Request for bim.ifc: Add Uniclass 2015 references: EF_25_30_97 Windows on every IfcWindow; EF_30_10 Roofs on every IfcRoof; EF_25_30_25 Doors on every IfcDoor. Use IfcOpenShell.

First a look at what the model holds.

```python
import ifcopenshell

model = ifcopenshell.open("bim.ifc")
print(model.schema)
print("classifications:", [c.Name for c in model.by_type("IfcClassification")])
for ifc_class in ("IfcDoor", "IfcRoof", "IfcStair", "IfcWall", "IfcWindow"):
    print(ifc_class, len(model.by_type(ifc_class)))
```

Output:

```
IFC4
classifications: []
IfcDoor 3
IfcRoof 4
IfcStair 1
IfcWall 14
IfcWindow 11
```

```python
import ifcopenshell
import ifcopenshell.api.classification

model = ifcopenshell.open("bim.ifc")

system = ifcopenshell.api.classification.add_classification(model, classification="Uniclass 2015")

codes = {
    "IfcWindow": ("EF_25_30_97", "Windows"),
    "IfcRoof": ("EF_30_10", "Roofs"),
    "IfcDoor": ("EF_25_30_25", "Doors"),
}
for ifc_class, (code, name) in codes.items():
    products = model.by_type(ifc_class)
    ifcopenshell.api.classification.add_reference(
        model, products=products, classification=system, identification=code, name=name
    )
    print(code, len(products))

model.write("bim-out.ifc")
```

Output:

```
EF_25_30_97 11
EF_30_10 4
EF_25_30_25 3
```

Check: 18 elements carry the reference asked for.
